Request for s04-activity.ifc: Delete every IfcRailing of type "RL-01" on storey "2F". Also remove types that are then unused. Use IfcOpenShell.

First a look at what the model holds.

```python
import ifcopenshell
import ifcopenshell.util.element

model = ifcopenshell.open("s04-activity.ifc")
print(model.schema)
storey = next(s for s in model.by_type("IfcBuildingStorey") if s.Name == "2F")
railings = [e for e in ifcopenshell.util.element.get_decomposition(storey) if e.is_a("IfcRailing")]
seen = {}
for e in railings:
    element_type = ifcopenshell.util.element.get_type(e)
    name = element_type.Name if element_type not in (None, e) else None
    seen[name] = seen.get(name, 0) + 1
for name, count in sorted(seen.items(), key=str):
    print(count, "x", name)
```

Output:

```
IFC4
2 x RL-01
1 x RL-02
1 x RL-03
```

```python
import ifcopenshell
import ifcopenshell.api.root
import ifcopenshell.util.element

model = ifcopenshell.open("s04-activity.ifc")

storey = next(s for s in model.by_type("IfcBuildingStorey") if s.Name == "2F")
railings = [e for e in ifcopenshell.util.element.get_decomposition(storey) if e.is_a("IfcRailing")]
targets = [e for e in railings if (t := ifcopenshell.util.element.get_type(e)) not in (None, e) and t.Name == "RL-01"]
types = {ifcopenshell.util.element.get_type(e) for e in targets} - {None, *targets}

for e in targets:
    ifcopenshell.api.root.remove_product(model, product=e)
print(len(targets), "removed")

unused = [t for t in types if not ifcopenshell.util.element.get_types(t)]
for t in unused:
    ifcopenshell.api.root.remove_product(model, product=t)
print(len(unused), "unused types removed")

model.write("s04-activity-out.ifc")
```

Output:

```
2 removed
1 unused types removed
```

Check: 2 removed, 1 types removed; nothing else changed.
